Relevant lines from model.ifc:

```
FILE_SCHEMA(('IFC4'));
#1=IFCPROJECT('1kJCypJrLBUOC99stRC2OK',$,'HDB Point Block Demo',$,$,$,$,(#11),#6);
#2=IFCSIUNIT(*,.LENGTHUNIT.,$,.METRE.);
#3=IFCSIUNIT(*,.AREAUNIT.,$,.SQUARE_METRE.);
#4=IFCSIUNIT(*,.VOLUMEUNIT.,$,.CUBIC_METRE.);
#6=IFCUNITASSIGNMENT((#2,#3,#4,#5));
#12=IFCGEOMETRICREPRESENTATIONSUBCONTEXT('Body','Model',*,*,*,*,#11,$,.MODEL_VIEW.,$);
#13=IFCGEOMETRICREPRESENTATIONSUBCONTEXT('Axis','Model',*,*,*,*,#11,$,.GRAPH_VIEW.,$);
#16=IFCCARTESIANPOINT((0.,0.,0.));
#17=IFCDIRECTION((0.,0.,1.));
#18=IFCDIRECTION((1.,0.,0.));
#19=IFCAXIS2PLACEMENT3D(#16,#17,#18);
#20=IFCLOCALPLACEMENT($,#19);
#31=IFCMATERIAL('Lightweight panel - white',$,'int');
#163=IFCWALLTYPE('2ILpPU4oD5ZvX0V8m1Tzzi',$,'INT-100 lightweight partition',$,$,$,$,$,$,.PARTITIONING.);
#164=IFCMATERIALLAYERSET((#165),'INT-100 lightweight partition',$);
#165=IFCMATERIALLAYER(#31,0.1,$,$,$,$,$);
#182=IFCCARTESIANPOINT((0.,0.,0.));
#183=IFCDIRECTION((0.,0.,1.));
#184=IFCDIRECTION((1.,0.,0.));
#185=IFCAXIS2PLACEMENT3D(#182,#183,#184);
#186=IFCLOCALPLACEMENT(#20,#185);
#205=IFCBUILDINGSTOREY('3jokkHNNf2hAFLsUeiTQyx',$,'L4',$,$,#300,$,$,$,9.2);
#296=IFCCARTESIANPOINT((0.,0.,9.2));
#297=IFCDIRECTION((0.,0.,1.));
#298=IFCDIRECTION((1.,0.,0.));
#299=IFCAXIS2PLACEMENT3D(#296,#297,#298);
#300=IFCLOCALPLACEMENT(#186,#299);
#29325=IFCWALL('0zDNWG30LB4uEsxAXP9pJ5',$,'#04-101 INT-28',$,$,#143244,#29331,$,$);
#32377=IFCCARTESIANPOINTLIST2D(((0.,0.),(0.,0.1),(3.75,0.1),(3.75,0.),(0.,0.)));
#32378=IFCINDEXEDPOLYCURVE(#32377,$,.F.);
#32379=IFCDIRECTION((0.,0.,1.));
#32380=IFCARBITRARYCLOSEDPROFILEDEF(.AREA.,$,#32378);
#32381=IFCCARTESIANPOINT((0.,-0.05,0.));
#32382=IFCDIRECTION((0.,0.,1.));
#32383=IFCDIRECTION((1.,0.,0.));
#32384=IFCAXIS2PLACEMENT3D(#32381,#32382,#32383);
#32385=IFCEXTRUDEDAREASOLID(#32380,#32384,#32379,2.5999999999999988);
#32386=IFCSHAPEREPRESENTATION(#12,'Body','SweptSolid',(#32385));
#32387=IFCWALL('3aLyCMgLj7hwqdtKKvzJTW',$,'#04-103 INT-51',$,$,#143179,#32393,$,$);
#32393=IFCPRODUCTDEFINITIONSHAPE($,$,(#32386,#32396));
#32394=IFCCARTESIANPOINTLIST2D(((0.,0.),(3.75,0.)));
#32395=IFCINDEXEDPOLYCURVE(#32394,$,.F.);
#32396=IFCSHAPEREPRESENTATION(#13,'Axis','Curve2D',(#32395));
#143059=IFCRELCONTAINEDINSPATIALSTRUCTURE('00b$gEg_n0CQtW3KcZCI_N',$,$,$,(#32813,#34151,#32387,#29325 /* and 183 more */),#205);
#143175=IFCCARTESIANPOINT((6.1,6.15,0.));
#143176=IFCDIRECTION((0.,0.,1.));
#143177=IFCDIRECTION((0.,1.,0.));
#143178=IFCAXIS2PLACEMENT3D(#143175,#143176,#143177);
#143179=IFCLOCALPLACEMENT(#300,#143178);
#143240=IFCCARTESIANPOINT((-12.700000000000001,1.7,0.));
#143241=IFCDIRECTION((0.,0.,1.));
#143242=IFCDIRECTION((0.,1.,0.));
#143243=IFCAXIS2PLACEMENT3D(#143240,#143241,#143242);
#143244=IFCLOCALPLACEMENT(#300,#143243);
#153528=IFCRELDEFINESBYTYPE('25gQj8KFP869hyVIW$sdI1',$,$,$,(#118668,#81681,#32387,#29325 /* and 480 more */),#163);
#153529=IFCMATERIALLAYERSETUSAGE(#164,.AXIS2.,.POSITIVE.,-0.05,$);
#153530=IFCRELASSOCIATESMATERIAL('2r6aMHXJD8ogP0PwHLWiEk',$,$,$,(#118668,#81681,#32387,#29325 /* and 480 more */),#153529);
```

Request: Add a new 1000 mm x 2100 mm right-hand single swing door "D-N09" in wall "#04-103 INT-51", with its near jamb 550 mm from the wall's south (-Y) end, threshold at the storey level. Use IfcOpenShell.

```python
import numpy as np
import ifcopenshell
import ifcopenshell.api.feature
import ifcopenshell.api.geometry
import ifcopenshell.api.root
import ifcopenshell.api.spatial
import ifcopenshell.geom
import ifcopenshell.util.element
import ifcopenshell.util.placement
import ifcopenshell.util.representation
import ifcopenshell.util.shape
import ifcopenshell.util.unit

model = ifcopenshell.open("model.ifc")
unit_scale = ifcopenshell.util.unit.calculate_unit_scale(model)
settings = ifcopenshell.geom.settings()


def volume(element):
    """Net volume in cubic metres, openings subtracted."""
    shape = ifcopenshell.geom.create_shape(settings, element)
    return ifcopenshell.util.shape.get_volume(shape.geometry)


wall = model.by_guid("3aLyCMgLj7hwqdtKKvzJTW")
storey = ifcopenshell.util.element.get_container(wall, ifc_class="IfcBuildingStorey")
context = ifcopenshell.util.representation.get_context(model, "Model", "Body", "MODEL_VIEW")
before = volume(wall)

width, height, from_end, sill = 1, 2.1, 0.55, 0.0  # metres

# The wall runs along its own X axis, and the end named is its -X end.
wall_shape = ifcopenshell.geom.create_shape(settings, wall)
x, y, z = ifcopenshell.util.shape.get_vertices(wall_shape.geometry).T
start = x.min() + from_end
face, thickness = float(y.min()), float(y.max() - y.min())
wall_matrix = ifcopenshell.util.placement.get_local_placement(wall.ObjectPlacement)
level = ifcopenshell.util.placement.get_local_placement(storey.ObjectPlacement)[2, 3]


def in_wall(x, y):
    """Placement at x, y metres in the wall's axes, at sill height."""
    matrix = wall_matrix.copy()
    matrix[:, 3] = wall_matrix @ np.array([x / unit_scale, y / unit_scale, 0.0, 1.0])
    matrix[2, 3] = level + sill / unit_scale
    return matrix


# Opening: a box that overshoots both wall faces by 50 mm.
opening = ifcopenshell.api.root.create_entity(model, ifc_class="IfcOpeningElement", predefined_type="OPENING")
box = ifcopenshell.api.geometry.add_wall_representation(
    model, context=context, length=width, height=height, thickness=thickness + 0.1
)
ifcopenshell.api.geometry.assign_representation(model, product=opening, representation=box)
ifcopenshell.api.geometry.edit_object_placement(model, product=opening, matrix=in_wall(start, face - 0.05), is_si=False)
ifcopenshell.api.feature.add_feature(model, feature=opening, element=wall)

door = ifcopenshell.api.root.create_entity(model, ifc_class="IfcDoor", name="D-N09", predefined_type="DOOR")
door.OverallWidth, door.OverallHeight = width / unit_scale, height / unit_scale
door.OperationType = "SINGLE_SWING_RIGHT"
body = ifcopenshell.api.geometry.add_door_representation(
    model,
    context=context,
    overall_width=door.OverallWidth,
    overall_height=door.OverallHeight,
    operation_type="SINGLE_SWING_RIGHT",
    lining_properties={"LiningDepth": thickness / unit_scale, "ThresholdDepth": thickness / unit_scale},
)
ifcopenshell.api.geometry.assign_representation(model, product=door, representation=body)
ifcopenshell.api.spatial.assign_container(model, products=[door], relating_structure=storey)
ifcopenshell.api.feature.add_filling(model, opening=opening, element=door)

# The lining spans the wall, so the door starts at the wall face.
ifcopenshell.api.geometry.edit_object_placement(model, product=door, matrix=in_wall(start, face), is_si=False)

after = volume(wall)

print(f"wall volume {before:.3f} -> {after:.3f} m3")

model.write("model_v2.ifc")
```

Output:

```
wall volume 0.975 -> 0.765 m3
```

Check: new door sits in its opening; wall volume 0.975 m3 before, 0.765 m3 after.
